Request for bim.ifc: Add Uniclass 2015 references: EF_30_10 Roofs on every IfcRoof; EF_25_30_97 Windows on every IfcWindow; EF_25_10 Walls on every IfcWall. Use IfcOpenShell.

First a look at what the model holds.

```python
import ifcopenshell

model = ifcopenshell.open("bim.ifc")
print(model.schema)
print("classifications:", [c.Name for c in model.by_type("IfcClassification")])
for ifc_class in ("IfcDoor", "IfcRoof", "IfcStair", "IfcWall", "IfcWindow"):
    print(ifc_class, len(model.by_type(ifc_class)))
```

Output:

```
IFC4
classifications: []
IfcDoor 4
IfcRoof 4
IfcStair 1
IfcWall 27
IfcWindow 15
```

```python
import ifcopenshell
import ifcopenshell.api.classification

model = ifcopenshell.open("bim.ifc")

system = ifcopenshell.api.classification.add_classification(model, classification="Uniclass 2015")

codes = {
    "IfcRoof": ("EF_30_10", "Roofs"),
    "IfcWindow": ("EF_25_30_97", "Windows"),
    "IfcWall": ("EF_25_10", "Walls"),
}
for ifc_class, (code, name) in codes.items():
    products = model.by_type(ifc_class)
    ifcopenshell.api.classification.add_reference(
        model, products=products, classification=system, identification=code, name=name
    )
    print(code, len(products))

model.write("bim_updated.ifc")
```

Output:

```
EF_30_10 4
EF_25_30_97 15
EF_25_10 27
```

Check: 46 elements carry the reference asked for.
